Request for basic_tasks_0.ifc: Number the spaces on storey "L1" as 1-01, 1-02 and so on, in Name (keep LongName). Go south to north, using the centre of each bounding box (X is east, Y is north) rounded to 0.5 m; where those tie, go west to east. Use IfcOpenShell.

First a look at what the model holds.

```python
import ifcopenshell
import ifcopenshell.util.element
import ifcopenshell.util.placement

model = ifcopenshell.open("basic_tasks_0.ifc")
print(model.schema)
storey = next(s for s in model.by_type("IfcBuildingStorey") if s.Name == "L1")
spaces = [e for e in ifcopenshell.util.element.get_decomposition(storey) if e.is_a("IfcSpace")]
for e in sorted(spaces, key=lambda e: e.id()):
    origin = ifcopenshell.util.placement.get_local_placement(e.ObjectPlacement)[:3, 3]
    print(e.id(), e.Name, e.LongName, origin.round(2) + 0.0, sep=" | ")
```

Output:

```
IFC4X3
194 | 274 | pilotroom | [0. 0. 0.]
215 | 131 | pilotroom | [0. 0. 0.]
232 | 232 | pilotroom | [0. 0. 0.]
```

```python
import ifcopenshell
import ifcopenshell.geom
import ifcopenshell.util.element
import ifcopenshell.util.shape

model = ifcopenshell.open("basic_tasks_0.ifc")
settings = ifcopenshell.geom.settings()
settings.set("use-world-coords", True)


def centre(element):
    shape = ifcopenshell.geom.create_shape(settings, element)
    return ifcopenshell.util.shape.get_bbox_centroid(shape.geometry)


storey = next(s for s in model.by_type("IfcBuildingStorey") if s.Name == "L1")
spaces = [e for e in ifcopenshell.util.element.get_decomposition(storey) if e.is_a("IfcSpace")]

# Insertion points can sit at a corner or the storey origin, so sort by the geometry (in metres).
centres = {e: centre(e) for e in spaces}
spaces.sort(key=lambda e: (round(centres[e][1] / 0.5), centres[e][0]))

for i, e in enumerate(spaces, start=1):
    number = f"1-{i:02d}"
    e.Name = number
    print(e.id(), number)

model.write("basic_tasks_0_updated.ifc")
```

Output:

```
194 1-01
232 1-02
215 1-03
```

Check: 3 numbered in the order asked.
